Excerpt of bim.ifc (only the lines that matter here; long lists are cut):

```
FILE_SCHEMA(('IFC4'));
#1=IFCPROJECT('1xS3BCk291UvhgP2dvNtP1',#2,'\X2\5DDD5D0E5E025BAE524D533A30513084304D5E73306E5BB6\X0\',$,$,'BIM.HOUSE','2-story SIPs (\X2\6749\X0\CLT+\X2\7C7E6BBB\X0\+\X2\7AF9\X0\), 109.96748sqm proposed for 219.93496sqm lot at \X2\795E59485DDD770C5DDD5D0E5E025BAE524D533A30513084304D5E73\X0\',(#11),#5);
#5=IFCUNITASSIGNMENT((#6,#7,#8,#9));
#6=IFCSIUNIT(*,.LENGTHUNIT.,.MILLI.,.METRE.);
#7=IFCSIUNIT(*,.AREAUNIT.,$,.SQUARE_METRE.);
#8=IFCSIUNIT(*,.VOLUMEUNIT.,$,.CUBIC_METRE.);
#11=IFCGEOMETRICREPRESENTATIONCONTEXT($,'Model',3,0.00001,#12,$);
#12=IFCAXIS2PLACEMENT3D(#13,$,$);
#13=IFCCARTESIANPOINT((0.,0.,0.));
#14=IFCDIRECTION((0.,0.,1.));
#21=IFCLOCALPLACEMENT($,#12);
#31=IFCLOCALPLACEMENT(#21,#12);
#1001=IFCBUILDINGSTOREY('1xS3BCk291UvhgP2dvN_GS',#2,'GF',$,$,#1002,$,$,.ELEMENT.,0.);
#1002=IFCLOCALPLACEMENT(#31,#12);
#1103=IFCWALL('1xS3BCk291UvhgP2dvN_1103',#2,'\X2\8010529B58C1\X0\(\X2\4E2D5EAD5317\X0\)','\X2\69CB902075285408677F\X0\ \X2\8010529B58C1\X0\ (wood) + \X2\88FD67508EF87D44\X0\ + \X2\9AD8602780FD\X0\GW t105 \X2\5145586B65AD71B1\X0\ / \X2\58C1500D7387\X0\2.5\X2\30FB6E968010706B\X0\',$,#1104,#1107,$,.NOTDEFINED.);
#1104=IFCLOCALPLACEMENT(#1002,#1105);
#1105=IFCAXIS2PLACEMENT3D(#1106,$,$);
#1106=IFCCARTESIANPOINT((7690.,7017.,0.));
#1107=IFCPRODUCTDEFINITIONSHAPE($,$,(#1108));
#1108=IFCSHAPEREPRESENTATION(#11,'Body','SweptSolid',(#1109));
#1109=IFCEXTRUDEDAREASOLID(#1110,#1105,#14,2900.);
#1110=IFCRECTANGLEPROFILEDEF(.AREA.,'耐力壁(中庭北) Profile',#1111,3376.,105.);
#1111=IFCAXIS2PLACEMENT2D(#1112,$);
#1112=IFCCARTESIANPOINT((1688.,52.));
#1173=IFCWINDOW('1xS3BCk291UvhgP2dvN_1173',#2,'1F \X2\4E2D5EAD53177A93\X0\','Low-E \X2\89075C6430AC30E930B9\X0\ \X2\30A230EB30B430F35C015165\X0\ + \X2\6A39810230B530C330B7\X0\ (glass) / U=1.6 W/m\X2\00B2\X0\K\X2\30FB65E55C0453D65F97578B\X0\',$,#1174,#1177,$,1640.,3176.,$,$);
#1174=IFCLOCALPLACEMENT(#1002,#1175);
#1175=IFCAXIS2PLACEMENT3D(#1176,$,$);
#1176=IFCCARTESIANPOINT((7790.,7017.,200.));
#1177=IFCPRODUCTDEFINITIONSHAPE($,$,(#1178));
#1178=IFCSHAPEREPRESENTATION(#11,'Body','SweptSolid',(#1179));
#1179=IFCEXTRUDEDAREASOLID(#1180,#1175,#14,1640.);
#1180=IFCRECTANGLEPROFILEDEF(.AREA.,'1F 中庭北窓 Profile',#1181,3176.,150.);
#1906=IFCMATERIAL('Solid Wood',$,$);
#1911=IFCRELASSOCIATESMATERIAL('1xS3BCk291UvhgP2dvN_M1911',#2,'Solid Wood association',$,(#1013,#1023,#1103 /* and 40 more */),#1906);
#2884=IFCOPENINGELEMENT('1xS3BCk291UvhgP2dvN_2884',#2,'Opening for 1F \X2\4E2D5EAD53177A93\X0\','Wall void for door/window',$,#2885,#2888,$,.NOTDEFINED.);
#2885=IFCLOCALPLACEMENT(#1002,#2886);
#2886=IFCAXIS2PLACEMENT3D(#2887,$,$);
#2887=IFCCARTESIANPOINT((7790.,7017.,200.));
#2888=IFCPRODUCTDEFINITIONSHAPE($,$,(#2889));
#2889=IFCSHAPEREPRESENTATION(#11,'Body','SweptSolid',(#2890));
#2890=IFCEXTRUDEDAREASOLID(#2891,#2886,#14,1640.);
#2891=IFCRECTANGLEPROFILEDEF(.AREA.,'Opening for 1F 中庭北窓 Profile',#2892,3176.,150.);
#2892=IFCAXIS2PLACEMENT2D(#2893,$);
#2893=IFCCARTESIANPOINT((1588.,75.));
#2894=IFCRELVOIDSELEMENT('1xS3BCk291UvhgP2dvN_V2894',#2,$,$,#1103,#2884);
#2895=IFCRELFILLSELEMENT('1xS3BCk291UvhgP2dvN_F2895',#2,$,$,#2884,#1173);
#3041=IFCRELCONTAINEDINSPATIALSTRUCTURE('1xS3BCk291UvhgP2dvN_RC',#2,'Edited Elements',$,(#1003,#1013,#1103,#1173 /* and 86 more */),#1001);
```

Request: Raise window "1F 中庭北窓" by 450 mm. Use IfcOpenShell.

```python
import numpy as np
import ifcopenshell
import ifcopenshell.api.geometry
import ifcopenshell.util.placement
import ifcopenshell.util.unit

model = ifcopenshell.open("bim.ifc")
unit_scale = ifcopenshell.util.unit.calculate_unit_scale(model)

window = model.by_id(1173)
opening = window.FillsVoids[0].RelatingOpeningElement
dz = 450.0

shift = np.array([0.0, 0.0, dz])
# The window is not placed relative to its opening, so move both.
for product in (opening, window):
    matrix = ifcopenshell.util.placement.get_local_placement(product.ObjectPlacement)
    matrix[:3, 3] += shift
    ifcopenshell.api.geometry.edit_object_placement(model, product=product, matrix=matrix, is_si=False)

print(f"moved by {dz * unit_scale:+.3f} m")

model.write("bim_edited.ifc")
```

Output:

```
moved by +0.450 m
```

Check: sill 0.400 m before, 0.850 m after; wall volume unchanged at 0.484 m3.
